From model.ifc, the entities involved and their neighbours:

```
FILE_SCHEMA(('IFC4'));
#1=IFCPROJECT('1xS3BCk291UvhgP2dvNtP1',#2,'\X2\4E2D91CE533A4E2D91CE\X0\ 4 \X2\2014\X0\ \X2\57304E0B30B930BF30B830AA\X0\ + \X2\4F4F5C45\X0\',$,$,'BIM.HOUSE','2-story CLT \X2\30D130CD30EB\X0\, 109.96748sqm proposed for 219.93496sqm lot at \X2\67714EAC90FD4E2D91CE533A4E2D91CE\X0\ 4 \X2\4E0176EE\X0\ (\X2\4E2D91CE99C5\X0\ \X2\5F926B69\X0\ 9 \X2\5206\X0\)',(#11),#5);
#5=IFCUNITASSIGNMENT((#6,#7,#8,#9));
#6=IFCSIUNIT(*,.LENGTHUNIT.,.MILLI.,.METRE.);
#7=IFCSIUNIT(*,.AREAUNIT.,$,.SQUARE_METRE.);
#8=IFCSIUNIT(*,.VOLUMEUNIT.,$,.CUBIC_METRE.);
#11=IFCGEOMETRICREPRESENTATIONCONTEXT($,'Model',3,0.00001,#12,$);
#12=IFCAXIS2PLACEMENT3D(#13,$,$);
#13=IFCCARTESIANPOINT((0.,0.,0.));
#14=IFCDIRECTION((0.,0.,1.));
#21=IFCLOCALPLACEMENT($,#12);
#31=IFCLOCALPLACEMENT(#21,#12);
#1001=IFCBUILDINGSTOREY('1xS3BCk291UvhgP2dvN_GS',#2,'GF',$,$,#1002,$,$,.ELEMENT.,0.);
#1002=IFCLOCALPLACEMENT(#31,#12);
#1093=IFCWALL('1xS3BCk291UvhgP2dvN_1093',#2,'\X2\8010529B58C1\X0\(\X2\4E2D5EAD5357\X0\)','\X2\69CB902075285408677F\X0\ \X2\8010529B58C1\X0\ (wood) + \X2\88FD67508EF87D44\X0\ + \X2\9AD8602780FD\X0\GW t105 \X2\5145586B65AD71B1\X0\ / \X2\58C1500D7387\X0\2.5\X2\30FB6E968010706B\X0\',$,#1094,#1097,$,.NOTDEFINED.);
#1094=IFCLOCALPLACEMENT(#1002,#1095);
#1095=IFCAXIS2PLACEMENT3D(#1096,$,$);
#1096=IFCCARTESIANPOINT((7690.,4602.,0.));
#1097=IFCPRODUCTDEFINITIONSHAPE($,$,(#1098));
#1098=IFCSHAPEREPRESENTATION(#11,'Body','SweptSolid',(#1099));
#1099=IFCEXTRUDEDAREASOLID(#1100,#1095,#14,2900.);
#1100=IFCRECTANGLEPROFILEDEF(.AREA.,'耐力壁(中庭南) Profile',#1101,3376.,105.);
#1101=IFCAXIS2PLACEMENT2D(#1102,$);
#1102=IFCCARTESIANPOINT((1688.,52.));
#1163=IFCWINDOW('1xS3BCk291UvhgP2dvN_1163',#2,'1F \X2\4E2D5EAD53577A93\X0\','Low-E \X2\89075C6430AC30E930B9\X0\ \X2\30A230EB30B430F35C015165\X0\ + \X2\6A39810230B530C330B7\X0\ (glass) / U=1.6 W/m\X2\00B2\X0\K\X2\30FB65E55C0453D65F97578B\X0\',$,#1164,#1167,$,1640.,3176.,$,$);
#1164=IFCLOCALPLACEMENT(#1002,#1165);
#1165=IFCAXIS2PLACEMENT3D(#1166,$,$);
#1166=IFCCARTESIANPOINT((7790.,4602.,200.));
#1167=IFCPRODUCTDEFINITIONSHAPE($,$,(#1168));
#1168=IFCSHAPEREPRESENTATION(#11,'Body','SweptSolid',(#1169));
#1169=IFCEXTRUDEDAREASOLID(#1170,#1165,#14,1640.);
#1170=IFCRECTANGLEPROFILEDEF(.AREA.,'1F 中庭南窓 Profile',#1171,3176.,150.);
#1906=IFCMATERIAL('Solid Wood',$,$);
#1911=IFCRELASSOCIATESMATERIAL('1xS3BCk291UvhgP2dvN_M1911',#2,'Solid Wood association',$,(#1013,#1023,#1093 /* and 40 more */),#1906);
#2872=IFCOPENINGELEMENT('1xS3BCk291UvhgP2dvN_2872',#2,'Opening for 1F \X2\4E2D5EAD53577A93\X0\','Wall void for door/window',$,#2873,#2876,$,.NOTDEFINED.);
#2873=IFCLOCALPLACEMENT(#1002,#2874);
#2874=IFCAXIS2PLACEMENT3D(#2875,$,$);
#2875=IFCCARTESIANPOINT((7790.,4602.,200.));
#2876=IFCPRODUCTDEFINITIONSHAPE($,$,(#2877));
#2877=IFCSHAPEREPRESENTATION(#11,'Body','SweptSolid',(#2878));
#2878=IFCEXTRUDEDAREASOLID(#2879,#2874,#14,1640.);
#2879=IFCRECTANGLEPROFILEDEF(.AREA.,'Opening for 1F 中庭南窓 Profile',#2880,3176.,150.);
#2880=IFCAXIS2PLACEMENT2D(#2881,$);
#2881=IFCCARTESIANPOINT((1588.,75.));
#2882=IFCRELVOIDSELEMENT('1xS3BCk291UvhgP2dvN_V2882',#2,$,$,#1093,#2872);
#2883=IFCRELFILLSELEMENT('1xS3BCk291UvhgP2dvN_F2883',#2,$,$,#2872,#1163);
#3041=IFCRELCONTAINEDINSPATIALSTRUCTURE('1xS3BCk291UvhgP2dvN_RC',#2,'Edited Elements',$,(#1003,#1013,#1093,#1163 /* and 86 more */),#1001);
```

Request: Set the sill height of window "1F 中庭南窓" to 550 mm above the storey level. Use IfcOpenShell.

```python
import numpy as np
import ifcopenshell
import ifcopenshell.api.geometry
import ifcopenshell.geom
import ifcopenshell.util.element
import ifcopenshell.util.placement
import ifcopenshell.util.shape
import ifcopenshell.util.unit

model = ifcopenshell.open("model.ifc")
unit_scale = ifcopenshell.util.unit.calculate_unit_scale(model)

window = model.by_guid("1xS3BCk291UvhgP2dvN_1163")
opening = window.FillsVoids[0].RelatingOpeningElement
storey = ifcopenshell.util.element.get_container(window, ifc_class="IfcBuildingStorey")
level = ifcopenshell.util.placement.get_local_placement(storey.ObjectPlacement)[2, 3]

# The opening's origin need not be at the sill, so measure its lowest point.
shape = ifcopenshell.geom.create_shape(ifcopenshell.geom.settings(), opening)
bottom = ifcopenshell.util.shape.get_shape_bottom_elevation(shape, shape.geometry) / unit_scale
dz = level + 0.55 / unit_scale - bottom

shift = np.array([0.0, 0.0, dz])
# The window is not placed relative to its opening, so move both.
for product in (opening, window):
    matrix = ifcopenshell.util.placement.get_local_placement(product.ObjectPlacement)
    matrix[:3, 3] += shift
    ifcopenshell.api.geometry.edit_object_placement(model, product=product, matrix=matrix, is_si=False)

print(f"moved by {dz * unit_scale:+.3f} m")

model.write("model_updated.ifc")
```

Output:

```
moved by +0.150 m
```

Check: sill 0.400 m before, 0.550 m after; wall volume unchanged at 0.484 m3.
